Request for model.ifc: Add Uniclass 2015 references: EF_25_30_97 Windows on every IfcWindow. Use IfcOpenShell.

First a look at what the model holds.

```python
import ifcopenshell

model = ifcopenshell.open("model.ifc")
print(model.schema)
print("classifications:", [c.Name for c in model.by_type("IfcClassification")])
for ifc_class in ("IfcDoor", "IfcRoof", "IfcStair", "IfcWall", "IfcWindow"):
    print(ifc_class, len(model.by_type(ifc_class)))
```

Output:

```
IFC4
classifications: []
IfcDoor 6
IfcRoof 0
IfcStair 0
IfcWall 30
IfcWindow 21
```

```python
import ifcopenshell
import ifcopenshell.api.classification

model = ifcopenshell.open("model.ifc")

system = ifcopenshell.api.classification.add_classification(model, classification="Uniclass 2015")

codes = {
    "IfcWindow": ("EF_25_30_97", "Windows"),
}
for ifc_class, (code, name) in codes.items():
    products = model.by_type(ifc_class)
    ifcopenshell.api.classification.add_reference(
        model, products=products, classification=system, identification=code, name=name
    )
    print(code, len(products))

model.write("model_rev.ifc")
```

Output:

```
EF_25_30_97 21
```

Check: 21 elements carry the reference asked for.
